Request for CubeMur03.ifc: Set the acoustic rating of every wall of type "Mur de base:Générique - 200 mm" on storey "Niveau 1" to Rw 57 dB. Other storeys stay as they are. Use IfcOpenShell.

First a look at what the model holds.

```python
import ifcopenshell
import ifcopenshell.util.element

model = ifcopenshell.open("CubeMur03.ifc")
print(model.schema)
storey = next(s for s in model.by_type("IfcBuildingStorey") if s.Name == "Niveau 1")
walls = [e for e in ifcopenshell.util.element.get_decomposition(storey) if e.is_a("IfcWall")]
seen = {}
for e in walls:
    element_type = ifcopenshell.util.element.get_type(e)
    key = (element_type.Name if element_type != e and element_type else None, ifcopenshell.util.element.get_pset(e, "Pset_WallCommon", "AcousticRating"))
    seen[key] = seen.get(key, 0) + 1
for (name, value), count in sorted(seen.items(), key=str):
    print(count, "x", name, "|", value)
```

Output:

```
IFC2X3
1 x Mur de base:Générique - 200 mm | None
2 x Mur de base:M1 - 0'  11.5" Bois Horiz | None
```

```python
import ifcopenshell
import ifcopenshell.api.pset
import ifcopenshell.util.element

model = ifcopenshell.open("CubeMur03.ifc")

storey = next(s for s in model.by_type("IfcBuildingStorey") if s.Name == "Niveau 1")
walls = [e for e in ifcopenshell.util.element.get_decomposition(storey) if e.is_a("IfcWall")]

count = 0
for e in walls:
    element_type = ifcopenshell.util.element.get_type(e)
    if element_type in (None, e) or element_type.Name != "Mur de base:Générique - 200 mm":
        continue
    # add_pset returns the element's existing set when there is one.
    pset = ifcopenshell.api.pset.add_pset(model, product=e, name="Pset_WallCommon")
    ifcopenshell.api.pset.edit_pset(model, pset=pset, properties={"AcousticRating": "Rw 57 dB"})
    count += 1

print(count, "walls updated")

model.write("CubeMur03_edited.ifc")
```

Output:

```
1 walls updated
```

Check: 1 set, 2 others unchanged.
